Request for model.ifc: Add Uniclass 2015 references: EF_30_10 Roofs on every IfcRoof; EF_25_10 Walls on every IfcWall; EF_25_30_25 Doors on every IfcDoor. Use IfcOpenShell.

First a look at what the model holds.

```python
import ifcopenshell

model = ifcopenshell.open("model.ifc")
print(model.schema)
print("classifications:", [c.Name for c in model.by_type("IfcClassification")])
for ifc_class in ("IfcDoor", "IfcRoof", "IfcStair", "IfcWall", "IfcWindow"):
    print(ifc_class, len(model.by_type(ifc_class)))
```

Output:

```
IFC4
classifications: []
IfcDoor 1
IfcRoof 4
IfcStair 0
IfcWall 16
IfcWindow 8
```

```python
import ifcopenshell
import ifcopenshell.api.classification

model = ifcopenshell.open("model.ifc")

system = ifcopenshell.api.classification.add_classification(model, classification="Uniclass 2015")

codes = {
    "IfcRoof": ("EF_30_10", "Roofs"),
    "IfcWall": ("EF_25_10", "Walls"),
    "IfcDoor": ("EF_25_30_25", "Doors"),
}
for ifc_class, (code, name) in codes.items():
    products = model.by_type(ifc_class)
    ifcopenshell.api.classification.add_reference(
        model, products=products, classification=system, identification=code, name=name
    )
    print(code, len(products))

model.write("model_v2.ifc")
```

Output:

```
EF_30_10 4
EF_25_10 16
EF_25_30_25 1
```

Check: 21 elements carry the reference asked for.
